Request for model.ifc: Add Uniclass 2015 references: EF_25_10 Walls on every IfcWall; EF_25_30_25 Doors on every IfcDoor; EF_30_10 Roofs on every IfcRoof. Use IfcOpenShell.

First a look at what the model holds.

```python
import ifcopenshell

model = ifcopenshell.open("model.ifc")
print(model.schema)
print("classifications:", [c.Name for c in model.by_type("IfcClassification")])
for ifc_class in ("IfcDoor", "IfcRoof", "IfcStair", "IfcWall", "IfcWindow"):
    print(ifc_class, len(model.by_type(ifc_class)))
```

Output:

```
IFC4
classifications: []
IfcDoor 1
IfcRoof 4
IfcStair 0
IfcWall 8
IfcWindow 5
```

```python
import ifcopenshell
import ifcopenshell.api.classification

model = ifcopenshell.open("model.ifc")

system = ifcopenshell.api.classification.add_classification(model, classification="Uniclass 2015")

codes = {
    "IfcWall": ("EF_25_10", "Walls"),
    "IfcDoor": ("EF_25_30_25", "Doors"),
    "IfcRoof": ("EF_30_10", "Roofs"),
}
for ifc_class, (code, name) in codes.items():
    products = model.by_type(ifc_class)
    ifcopenshell.api.classification.add_reference(
        model, products=products, classification=system, identification=code, name=name
    )
    print(code, len(products))

model.write("model_rev.ifc")
```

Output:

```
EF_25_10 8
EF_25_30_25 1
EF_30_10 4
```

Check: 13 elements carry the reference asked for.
